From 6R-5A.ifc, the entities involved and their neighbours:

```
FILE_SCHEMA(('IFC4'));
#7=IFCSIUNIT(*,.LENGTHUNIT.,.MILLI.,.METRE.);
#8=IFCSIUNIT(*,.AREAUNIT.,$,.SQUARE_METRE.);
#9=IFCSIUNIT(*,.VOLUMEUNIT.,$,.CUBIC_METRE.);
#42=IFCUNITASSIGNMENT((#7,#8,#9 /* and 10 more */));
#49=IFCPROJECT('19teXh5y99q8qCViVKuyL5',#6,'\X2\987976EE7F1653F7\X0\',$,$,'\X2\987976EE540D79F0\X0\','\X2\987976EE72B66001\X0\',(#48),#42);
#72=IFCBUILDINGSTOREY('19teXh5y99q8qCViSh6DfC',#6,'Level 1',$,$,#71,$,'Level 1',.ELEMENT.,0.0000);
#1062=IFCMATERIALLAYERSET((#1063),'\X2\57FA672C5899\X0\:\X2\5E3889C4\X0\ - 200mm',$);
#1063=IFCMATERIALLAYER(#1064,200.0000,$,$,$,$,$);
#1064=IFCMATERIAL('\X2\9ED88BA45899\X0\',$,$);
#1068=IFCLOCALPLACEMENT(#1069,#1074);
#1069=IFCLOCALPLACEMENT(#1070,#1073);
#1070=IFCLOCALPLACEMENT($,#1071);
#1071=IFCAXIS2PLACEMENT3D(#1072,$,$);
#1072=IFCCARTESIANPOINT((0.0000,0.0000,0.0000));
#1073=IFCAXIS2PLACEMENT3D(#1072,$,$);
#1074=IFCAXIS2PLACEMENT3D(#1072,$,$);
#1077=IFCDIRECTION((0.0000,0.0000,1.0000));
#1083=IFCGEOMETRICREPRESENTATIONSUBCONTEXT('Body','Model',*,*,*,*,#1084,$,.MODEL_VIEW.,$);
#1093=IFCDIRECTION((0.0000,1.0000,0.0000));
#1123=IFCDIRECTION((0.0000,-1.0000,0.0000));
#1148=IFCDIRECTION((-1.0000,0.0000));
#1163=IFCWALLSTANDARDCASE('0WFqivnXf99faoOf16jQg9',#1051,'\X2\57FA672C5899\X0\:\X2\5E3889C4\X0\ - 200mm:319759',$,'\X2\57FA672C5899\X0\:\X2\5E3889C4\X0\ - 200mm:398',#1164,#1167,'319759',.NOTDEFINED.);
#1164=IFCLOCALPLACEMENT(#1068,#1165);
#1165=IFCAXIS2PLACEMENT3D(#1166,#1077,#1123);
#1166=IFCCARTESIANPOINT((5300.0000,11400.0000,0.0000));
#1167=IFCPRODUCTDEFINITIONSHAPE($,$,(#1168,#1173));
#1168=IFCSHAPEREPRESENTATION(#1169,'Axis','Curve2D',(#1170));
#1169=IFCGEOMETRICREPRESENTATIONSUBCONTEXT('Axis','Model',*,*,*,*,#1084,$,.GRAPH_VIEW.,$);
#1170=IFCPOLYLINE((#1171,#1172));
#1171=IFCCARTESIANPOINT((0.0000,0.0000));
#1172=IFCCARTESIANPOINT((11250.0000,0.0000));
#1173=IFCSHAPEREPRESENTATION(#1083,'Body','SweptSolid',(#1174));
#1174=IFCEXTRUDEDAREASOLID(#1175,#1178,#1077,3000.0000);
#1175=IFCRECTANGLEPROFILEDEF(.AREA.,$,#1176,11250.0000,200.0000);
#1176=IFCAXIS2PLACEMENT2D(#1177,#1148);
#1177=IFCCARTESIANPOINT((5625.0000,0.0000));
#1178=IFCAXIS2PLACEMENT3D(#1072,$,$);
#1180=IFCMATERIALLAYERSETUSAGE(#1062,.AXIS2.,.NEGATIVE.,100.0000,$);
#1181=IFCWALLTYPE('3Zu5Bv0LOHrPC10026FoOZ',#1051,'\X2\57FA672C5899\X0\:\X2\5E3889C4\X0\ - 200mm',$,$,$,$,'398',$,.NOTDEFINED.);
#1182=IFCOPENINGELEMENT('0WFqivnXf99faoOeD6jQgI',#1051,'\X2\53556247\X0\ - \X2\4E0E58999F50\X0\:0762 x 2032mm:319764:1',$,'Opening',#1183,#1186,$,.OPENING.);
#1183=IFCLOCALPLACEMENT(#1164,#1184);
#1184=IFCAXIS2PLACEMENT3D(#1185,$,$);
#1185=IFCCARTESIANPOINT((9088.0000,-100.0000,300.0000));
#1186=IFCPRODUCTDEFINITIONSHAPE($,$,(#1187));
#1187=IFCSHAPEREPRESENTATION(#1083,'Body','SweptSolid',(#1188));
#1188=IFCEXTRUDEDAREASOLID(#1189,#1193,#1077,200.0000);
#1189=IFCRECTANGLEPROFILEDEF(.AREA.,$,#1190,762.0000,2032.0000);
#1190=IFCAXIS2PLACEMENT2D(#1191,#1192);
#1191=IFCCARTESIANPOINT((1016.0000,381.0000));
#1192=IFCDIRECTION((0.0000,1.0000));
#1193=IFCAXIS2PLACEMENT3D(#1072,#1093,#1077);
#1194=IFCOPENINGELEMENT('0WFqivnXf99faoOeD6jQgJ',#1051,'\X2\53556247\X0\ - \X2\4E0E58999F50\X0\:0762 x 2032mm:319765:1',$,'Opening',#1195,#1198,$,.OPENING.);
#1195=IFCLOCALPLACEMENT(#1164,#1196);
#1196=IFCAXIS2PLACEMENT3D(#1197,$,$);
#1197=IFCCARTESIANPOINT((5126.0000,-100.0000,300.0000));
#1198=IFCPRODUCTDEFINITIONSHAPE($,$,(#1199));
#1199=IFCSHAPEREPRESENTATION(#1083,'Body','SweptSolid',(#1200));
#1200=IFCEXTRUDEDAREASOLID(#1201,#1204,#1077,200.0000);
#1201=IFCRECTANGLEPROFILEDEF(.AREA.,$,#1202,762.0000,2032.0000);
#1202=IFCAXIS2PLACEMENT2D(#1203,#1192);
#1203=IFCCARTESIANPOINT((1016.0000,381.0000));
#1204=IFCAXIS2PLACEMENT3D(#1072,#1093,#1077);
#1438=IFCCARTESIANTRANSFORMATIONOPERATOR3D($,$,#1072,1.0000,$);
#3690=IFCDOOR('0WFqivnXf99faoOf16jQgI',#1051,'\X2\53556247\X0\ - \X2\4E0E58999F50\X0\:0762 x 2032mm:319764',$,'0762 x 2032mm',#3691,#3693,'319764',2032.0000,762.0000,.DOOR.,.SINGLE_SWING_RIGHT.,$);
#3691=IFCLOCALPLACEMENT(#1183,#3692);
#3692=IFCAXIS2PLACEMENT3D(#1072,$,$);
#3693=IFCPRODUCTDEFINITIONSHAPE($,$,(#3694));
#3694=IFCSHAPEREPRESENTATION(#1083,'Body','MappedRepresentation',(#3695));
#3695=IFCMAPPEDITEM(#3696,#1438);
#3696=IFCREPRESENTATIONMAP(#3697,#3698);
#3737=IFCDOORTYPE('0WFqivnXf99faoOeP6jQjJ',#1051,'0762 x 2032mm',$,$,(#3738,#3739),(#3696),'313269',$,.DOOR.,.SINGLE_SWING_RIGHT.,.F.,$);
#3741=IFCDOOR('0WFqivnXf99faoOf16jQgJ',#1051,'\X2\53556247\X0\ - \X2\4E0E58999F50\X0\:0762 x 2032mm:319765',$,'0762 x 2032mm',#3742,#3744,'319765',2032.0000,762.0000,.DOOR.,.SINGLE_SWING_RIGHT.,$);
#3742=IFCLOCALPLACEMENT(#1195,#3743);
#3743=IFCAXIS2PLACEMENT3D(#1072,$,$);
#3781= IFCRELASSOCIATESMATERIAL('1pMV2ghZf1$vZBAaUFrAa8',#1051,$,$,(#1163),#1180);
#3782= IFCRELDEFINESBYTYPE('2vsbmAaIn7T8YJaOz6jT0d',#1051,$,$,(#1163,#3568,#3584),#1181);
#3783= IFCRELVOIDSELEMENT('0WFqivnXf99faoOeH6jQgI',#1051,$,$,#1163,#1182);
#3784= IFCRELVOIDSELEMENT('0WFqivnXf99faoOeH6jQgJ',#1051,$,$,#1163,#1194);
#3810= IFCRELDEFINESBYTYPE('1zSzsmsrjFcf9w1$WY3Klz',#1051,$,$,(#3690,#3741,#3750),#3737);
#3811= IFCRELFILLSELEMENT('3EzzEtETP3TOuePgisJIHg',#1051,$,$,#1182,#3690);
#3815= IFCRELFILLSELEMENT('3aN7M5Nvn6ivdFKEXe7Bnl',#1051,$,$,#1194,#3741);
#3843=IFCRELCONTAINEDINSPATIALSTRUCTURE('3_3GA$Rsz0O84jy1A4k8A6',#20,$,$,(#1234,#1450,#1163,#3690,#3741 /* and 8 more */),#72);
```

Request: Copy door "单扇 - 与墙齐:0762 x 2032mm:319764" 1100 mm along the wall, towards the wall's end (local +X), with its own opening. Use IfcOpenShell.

```python
import ifcopenshell
import ifcopenshell.api.feature
import ifcopenshell.api.geometry
import ifcopenshell.api.root
import ifcopenshell.geom
import ifcopenshell.util.element
import ifcopenshell.util.placement
import ifcopenshell.util.shape
import ifcopenshell.util.unit

model = ifcopenshell.open("6R-5A.ifc")
unit_scale = ifcopenshell.util.unit.calculate_unit_scale(model)
settings = ifcopenshell.geom.settings()


def volume(element):
    """Net volume in cubic metres, openings subtracted."""
    shape = ifcopenshell.geom.create_shape(settings, element)
    return ifcopenshell.util.shape.get_volume(shape.geometry)


def reuse_history(source, copy):
    """copy_class also copies each property set's owner history, people and application; keep the originals."""
    for rel in copy.IsDefinedBy:
        if rel.is_a("IfcRelDefinesByProperties") and (history := rel.RelatingPropertyDefinition.OwnerHistory):
            rel.RelatingPropertyDefinition.OwnerHistory = source.OwnerHistory
            ifcopenshell.util.element.remove_deep2(model, history)


door = model.by_guid("0WFqivnXf99faoOf16jQgI")
opening = door.FillsVoids[0].RelatingOpeningElement
wall = opening.VoidsElements[0].RelatingBuildingElement
before = volume(wall)
shift = ifcopenshell.util.placement.get_local_placement(wall.ObjectPlacement)[:3, 0] * 1.1 / unit_scale

# copy_class copies the void relationship, type, container and properties, but no geometry.
new_opening = ifcopenshell.api.root.copy_class(model, product=opening)
new_opening.Representation = ifcopenshell.util.element.copy_deep(
    model, opening.Representation, exclude=["IfcGeometricRepresentationContext", "IfcRepresentationMap"]
)
new_opening.Name = "单扇 - 与墙齐:0762 x 2032mm"
new_door = ifcopenshell.api.root.copy_class(model, product=door)
new_door.Representation = ifcopenshell.util.element.copy_deep(
    model, door.Representation, exclude=["IfcGeometricRepresentationContext", "IfcRepresentationMap"]
)
new_door.Name = "单扇 - 与墙齐:0762 x 2032mm"
new_door.Tag = None
reuse_history(door, new_door)
ifcopenshell.api.feature.add_filling(model, opening=new_opening, element=new_door)

for old, new in ((opening, new_opening), (door, new_door)):
    matrix = ifcopenshell.util.placement.get_local_placement(old.ObjectPlacement)
    matrix[:3, 3] += shift
    ifcopenshell.api.geometry.edit_object_placement(model, product=new, matrix=matrix, is_si=False)

after = volume(wall)

print(f"wall volume {before:.3f} -> {after:.3f} m3")

model.write("6R-5A_updated.ifc")
```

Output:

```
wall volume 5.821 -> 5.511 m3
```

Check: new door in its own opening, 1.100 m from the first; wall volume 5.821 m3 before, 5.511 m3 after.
